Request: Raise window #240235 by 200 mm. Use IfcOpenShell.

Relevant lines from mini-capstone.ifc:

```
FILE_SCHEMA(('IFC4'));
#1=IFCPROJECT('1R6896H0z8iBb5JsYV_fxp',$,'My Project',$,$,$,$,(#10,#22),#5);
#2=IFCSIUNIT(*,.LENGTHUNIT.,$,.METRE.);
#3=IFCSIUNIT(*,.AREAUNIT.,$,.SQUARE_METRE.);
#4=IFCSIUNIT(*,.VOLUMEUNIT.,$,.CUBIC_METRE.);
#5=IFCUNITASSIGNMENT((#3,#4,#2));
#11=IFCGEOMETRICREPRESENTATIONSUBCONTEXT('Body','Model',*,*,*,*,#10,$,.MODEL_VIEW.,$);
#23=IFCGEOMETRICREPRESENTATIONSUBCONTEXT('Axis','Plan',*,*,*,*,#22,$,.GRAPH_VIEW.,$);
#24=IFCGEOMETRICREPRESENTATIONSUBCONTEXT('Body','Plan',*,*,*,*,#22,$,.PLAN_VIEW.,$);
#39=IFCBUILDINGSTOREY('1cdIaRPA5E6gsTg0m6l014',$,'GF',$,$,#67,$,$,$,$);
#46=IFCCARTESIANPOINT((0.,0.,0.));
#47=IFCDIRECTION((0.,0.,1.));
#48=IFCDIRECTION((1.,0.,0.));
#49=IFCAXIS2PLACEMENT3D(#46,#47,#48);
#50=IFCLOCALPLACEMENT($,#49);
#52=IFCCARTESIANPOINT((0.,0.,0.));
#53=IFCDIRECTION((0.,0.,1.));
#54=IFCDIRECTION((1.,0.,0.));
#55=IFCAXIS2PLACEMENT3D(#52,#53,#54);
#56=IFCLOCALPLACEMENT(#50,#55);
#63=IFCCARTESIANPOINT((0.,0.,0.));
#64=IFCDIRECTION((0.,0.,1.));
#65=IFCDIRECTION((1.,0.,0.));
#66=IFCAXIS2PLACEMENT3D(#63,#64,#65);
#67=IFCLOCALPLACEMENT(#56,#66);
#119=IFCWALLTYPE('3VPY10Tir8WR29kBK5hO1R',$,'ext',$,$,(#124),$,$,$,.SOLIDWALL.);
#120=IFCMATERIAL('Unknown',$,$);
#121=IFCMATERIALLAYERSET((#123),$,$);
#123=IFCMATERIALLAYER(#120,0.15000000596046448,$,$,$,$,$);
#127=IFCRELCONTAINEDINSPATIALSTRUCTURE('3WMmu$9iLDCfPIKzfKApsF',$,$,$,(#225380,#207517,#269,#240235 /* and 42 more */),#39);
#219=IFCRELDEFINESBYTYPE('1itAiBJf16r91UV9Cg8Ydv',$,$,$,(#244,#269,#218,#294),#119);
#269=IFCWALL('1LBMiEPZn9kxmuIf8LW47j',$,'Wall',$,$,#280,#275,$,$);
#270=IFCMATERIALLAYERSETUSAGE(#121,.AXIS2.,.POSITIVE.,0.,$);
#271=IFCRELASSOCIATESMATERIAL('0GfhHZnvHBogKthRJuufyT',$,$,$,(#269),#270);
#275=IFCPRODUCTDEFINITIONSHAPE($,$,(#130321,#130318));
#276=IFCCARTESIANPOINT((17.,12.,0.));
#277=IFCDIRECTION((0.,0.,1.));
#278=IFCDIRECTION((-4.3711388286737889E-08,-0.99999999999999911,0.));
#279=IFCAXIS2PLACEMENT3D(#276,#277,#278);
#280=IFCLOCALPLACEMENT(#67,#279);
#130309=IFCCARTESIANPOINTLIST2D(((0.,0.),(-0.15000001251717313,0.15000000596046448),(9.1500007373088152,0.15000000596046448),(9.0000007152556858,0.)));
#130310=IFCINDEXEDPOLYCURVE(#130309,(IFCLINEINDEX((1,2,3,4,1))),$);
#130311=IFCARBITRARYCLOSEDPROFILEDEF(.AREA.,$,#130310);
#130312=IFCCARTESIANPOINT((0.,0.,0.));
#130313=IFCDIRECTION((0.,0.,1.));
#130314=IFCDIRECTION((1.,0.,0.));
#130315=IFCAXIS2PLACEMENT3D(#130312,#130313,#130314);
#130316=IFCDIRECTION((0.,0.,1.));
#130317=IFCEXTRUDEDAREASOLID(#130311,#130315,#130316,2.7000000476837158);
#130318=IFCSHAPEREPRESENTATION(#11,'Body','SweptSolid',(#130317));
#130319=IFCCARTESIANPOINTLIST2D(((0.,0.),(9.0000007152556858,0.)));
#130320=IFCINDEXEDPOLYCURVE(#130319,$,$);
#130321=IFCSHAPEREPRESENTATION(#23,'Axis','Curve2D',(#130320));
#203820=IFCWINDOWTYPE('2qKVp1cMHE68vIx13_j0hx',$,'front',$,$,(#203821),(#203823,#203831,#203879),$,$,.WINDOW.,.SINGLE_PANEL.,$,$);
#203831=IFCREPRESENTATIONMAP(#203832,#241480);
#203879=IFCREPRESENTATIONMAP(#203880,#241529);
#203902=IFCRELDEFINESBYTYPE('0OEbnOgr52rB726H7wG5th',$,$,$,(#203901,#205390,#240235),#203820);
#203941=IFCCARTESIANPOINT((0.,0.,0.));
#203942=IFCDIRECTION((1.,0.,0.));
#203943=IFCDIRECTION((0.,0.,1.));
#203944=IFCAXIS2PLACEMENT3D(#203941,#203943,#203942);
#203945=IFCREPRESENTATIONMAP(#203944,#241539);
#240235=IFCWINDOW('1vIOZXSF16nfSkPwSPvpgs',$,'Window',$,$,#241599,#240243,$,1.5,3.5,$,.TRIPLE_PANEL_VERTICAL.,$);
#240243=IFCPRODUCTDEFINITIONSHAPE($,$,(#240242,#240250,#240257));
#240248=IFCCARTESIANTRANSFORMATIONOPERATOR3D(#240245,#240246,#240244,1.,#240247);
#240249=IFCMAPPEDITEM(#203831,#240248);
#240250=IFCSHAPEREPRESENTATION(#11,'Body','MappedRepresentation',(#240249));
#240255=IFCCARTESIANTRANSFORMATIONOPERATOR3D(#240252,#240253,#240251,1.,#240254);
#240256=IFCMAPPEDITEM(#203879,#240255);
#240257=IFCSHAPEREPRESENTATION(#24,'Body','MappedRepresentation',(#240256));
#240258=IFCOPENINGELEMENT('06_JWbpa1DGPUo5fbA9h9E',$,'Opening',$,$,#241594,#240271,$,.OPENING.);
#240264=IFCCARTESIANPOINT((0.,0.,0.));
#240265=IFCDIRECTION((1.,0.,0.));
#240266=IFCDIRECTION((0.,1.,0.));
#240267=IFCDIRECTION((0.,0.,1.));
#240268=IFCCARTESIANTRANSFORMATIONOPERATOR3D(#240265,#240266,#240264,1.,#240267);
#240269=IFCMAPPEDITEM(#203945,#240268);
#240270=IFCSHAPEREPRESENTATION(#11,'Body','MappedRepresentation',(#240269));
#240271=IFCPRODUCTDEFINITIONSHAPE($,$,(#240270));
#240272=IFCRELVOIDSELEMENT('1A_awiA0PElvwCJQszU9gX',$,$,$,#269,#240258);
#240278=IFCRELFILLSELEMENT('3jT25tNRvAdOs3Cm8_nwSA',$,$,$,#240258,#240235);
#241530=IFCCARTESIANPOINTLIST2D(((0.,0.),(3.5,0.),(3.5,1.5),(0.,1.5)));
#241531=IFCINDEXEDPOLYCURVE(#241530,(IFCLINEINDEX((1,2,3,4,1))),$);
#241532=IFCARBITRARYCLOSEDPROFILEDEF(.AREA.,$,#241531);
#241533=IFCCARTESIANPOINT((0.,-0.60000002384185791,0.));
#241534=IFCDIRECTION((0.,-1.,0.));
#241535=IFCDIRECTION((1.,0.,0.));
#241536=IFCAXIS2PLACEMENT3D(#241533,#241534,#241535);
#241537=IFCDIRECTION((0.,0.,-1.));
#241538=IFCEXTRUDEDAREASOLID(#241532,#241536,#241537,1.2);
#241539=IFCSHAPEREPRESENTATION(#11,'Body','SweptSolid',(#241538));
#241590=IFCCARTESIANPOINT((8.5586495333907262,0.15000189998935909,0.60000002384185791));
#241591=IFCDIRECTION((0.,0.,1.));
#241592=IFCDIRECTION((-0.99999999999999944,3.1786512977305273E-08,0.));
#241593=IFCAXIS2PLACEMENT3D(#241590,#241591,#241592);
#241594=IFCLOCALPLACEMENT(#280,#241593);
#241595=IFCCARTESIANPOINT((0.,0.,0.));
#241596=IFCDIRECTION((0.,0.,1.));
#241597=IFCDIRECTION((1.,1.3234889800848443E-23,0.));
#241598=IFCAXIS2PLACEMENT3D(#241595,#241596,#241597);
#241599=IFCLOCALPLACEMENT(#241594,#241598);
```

```python
import numpy as np
import ifcopenshell
import ifcopenshell.api.geometry
import ifcopenshell.util.placement
import ifcopenshell.util.unit

model = ifcopenshell.open("mini-capstone.ifc")
unit_scale = ifcopenshell.util.unit.calculate_unit_scale(model)

window = model.by_id(240235)
opening = window.FillsVoids[0].RelatingOpeningElement
dz = 0.2 / unit_scale

shift = np.array([0.0, 0.0, dz])
# The window is placed relative to its opening, so it follows when the opening moves.
matrix = ifcopenshell.util.placement.get_local_placement(opening.ObjectPlacement)
matrix[:3, 3] += shift
ifcopenshell.api.geometry.edit_object_placement(
    model, product=opening, matrix=matrix, is_si=False, should_transform_children=True
)

print(f"moved by {dz * unit_scale:+.3f} m")

model.write("mini-capstone-out.ifc")
```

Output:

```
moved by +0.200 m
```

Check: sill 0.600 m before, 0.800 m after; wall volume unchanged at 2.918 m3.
